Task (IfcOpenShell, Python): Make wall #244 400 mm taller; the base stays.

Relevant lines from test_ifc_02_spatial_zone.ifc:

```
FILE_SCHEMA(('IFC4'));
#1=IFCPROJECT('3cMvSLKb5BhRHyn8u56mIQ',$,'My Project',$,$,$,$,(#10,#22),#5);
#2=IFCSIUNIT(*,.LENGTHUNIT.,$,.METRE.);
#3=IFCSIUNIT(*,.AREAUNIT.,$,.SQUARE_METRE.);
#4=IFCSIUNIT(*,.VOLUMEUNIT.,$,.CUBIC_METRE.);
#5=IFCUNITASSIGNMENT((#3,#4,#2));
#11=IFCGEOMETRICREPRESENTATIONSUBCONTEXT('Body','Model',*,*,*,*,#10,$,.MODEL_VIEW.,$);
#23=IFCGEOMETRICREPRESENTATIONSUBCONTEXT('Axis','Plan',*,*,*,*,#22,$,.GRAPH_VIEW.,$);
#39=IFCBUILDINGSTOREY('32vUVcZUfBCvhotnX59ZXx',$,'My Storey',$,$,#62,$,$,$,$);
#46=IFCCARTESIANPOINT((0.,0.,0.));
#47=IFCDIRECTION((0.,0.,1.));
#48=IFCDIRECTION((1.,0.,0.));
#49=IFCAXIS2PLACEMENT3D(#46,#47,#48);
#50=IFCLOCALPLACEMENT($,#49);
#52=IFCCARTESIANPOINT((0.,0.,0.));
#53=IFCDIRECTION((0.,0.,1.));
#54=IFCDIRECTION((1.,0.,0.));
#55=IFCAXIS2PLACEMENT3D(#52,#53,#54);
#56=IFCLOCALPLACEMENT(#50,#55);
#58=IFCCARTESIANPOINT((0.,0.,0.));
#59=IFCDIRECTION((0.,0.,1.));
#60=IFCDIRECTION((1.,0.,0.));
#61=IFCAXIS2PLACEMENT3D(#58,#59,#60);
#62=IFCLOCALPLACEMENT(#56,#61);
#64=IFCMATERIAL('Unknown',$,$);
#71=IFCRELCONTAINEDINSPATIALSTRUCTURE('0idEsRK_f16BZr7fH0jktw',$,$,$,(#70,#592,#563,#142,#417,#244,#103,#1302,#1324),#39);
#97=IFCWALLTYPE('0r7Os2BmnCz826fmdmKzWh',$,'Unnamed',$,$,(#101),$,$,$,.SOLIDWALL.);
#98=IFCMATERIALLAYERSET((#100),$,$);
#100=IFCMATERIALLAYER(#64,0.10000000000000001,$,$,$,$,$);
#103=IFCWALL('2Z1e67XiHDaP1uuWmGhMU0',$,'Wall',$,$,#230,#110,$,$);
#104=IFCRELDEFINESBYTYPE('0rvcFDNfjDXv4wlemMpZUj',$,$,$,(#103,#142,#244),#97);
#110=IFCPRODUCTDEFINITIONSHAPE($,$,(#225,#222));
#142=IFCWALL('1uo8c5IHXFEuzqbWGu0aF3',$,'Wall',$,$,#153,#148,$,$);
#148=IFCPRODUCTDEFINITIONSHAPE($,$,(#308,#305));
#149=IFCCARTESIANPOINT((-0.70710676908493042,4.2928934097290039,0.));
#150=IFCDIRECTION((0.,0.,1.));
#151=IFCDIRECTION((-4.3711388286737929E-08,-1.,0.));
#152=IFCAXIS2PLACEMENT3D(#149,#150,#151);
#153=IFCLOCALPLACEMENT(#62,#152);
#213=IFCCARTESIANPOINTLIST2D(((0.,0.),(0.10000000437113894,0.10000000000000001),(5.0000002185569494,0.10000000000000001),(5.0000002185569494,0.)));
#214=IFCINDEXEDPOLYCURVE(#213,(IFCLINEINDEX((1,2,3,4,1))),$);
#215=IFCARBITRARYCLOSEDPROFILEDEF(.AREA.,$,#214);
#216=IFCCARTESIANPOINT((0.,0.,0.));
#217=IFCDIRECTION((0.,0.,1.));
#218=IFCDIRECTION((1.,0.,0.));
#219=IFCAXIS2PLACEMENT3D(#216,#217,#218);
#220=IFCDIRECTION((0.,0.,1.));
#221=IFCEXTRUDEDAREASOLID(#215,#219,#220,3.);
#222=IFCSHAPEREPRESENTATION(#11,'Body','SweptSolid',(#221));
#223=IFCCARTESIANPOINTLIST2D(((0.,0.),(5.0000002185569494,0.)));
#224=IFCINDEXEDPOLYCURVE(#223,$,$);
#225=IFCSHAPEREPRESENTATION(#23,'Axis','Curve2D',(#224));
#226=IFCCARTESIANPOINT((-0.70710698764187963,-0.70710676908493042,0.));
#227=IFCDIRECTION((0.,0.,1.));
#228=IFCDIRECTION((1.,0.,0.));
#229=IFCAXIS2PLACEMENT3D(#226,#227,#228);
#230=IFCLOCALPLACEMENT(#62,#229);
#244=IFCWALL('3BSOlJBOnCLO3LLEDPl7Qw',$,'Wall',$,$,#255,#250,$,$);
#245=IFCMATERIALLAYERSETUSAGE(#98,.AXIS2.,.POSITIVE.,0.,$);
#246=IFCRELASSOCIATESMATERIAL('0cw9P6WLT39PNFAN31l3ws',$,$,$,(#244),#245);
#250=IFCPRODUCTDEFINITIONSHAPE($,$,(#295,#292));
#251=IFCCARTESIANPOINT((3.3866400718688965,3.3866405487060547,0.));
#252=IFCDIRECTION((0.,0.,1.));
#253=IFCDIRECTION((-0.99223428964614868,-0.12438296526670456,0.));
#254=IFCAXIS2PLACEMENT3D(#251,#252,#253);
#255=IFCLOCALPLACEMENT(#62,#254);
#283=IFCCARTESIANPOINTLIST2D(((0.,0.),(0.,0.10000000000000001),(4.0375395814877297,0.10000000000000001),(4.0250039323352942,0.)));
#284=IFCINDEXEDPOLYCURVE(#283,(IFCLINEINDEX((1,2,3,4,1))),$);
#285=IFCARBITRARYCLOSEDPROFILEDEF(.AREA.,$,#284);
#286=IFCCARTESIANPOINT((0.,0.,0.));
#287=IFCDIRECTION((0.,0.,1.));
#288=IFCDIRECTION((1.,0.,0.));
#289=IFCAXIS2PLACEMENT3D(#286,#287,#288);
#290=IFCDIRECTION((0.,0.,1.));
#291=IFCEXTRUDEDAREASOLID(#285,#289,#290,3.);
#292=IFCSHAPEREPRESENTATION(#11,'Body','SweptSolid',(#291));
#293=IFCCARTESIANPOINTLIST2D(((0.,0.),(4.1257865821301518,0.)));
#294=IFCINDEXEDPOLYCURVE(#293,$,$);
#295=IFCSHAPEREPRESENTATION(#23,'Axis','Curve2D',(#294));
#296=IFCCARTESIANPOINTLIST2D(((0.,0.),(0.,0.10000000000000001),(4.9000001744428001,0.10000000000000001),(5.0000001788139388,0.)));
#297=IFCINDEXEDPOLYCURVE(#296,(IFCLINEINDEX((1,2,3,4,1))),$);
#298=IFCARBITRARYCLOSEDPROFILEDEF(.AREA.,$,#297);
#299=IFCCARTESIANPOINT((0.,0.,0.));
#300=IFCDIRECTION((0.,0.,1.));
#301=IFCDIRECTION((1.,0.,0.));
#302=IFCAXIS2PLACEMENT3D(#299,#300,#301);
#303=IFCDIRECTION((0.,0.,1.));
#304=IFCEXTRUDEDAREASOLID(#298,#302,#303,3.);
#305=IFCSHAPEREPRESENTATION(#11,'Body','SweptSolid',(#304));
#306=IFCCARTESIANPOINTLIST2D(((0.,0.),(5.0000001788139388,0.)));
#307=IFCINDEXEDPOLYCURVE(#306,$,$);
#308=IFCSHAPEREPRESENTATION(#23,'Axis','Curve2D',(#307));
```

```python
import ifcopenshell
import ifcopenshell.geom
import ifcopenshell.util.representation
import ifcopenshell.util.shape

model = ifcopenshell.open("test_ifc_02_spatial_zone.ifc")
settings = ifcopenshell.geom.settings()


def volume(element):
    """Net volume in cubic metres, openings subtracted."""
    shape = ifcopenshell.geom.create_shape(settings, element)
    return ifcopenshell.util.shape.get_volume(shape.geometry)


wall = model.by_guid("3BSOlJBOnCLO3LLEDPl7Qw")
before = volume(wall)

body = ifcopenshell.util.representation.get_representation(wall, "Model", "Body")
solid = body.Items[0]
old_height = solid.Depth
solid.Depth += 0.4
after = volume(wall)

print(f"height {old_height:g} -> {solid.Depth:g}, volume {before:.3f} -> {after:.3f} m3")

model.write("test_ifc_02_spatial_zone_v2.ifc")
```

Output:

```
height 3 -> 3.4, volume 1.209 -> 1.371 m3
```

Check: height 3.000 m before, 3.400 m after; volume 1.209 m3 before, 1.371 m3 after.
